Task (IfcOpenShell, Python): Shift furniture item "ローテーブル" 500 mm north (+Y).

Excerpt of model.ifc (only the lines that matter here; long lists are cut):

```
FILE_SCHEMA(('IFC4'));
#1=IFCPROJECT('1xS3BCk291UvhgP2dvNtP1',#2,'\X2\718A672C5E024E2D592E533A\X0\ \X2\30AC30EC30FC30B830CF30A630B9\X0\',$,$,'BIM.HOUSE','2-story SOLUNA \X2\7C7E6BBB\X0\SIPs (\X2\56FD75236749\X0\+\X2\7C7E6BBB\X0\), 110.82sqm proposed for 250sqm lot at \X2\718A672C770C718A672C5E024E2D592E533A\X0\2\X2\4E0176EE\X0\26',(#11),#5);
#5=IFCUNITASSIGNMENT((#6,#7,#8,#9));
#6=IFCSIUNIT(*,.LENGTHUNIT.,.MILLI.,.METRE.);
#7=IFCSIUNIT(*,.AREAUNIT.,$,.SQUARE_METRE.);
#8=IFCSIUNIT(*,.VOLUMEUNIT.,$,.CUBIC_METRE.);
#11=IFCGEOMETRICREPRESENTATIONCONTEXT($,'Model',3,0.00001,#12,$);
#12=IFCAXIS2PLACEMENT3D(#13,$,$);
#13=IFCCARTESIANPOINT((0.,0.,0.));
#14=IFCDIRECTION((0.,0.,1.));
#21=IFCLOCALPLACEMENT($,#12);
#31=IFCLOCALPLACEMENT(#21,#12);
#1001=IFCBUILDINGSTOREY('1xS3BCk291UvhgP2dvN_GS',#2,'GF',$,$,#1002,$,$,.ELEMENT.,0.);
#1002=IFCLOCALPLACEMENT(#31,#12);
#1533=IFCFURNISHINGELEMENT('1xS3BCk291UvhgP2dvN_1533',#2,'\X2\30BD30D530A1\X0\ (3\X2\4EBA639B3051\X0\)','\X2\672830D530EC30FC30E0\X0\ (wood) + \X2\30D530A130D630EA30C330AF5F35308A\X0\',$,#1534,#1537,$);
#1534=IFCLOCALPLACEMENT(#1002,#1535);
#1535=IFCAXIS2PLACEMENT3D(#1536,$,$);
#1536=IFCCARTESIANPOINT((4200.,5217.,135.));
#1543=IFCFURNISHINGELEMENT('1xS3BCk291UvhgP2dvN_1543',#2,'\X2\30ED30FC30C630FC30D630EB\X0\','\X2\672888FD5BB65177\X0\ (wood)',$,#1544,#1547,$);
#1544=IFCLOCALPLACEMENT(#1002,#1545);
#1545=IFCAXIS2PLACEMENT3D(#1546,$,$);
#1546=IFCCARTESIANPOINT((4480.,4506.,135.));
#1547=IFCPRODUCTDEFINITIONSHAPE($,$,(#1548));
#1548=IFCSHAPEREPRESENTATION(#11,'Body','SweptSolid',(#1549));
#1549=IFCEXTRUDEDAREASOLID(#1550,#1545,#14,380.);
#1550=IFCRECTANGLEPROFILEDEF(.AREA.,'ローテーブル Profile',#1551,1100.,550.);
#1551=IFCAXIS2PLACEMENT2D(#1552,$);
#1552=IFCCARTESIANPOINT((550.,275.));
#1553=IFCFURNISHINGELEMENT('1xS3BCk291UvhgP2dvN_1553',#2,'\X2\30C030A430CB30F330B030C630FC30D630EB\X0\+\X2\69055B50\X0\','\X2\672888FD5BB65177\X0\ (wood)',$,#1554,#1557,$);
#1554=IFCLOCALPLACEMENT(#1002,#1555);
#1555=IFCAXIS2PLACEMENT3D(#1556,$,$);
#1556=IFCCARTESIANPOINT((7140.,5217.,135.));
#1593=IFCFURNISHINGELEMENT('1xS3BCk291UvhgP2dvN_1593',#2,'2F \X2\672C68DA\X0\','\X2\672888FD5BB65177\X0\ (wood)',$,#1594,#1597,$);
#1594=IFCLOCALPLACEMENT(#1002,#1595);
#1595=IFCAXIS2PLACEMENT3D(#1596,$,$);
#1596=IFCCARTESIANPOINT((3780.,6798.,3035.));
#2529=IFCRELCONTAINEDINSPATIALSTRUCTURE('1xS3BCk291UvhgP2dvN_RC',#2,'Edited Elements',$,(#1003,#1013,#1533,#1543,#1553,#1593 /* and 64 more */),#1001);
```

```python
import ifcopenshell
import ifcopenshell.api.geometry
import ifcopenshell.util.placement

model = ifcopenshell.open("model.ifc")

item = model.by_id(1543)
matrix = ifcopenshell.util.placement.get_local_placement(item.ObjectPlacement)
matrix[1, 3] += 500.0
ifcopenshell.api.geometry.edit_object_placement(model, product=item, matrix=matrix, is_si=False)

print(ifcopenshell.util.placement.get_local_placement(item.ObjectPlacement).round(3) + 0.0)

model.write("model_updated.ifc")
```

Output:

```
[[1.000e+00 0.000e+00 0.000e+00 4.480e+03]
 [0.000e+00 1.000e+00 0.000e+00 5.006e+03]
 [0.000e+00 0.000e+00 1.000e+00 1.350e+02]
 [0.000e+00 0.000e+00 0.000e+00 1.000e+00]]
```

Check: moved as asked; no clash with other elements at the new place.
